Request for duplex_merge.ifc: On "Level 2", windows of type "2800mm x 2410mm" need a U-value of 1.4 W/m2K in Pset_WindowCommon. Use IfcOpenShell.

First a look at what the model holds.

```python
import ifcopenshell
import ifcopenshell.util.element

model = ifcopenshell.open("duplex_merge.ifc")
print(model.schema)
storey = next(s for s in model.by_type("IfcBuildingStorey") if s.Name == "Level 2")
windows = [e for e in ifcopenshell.util.element.get_decomposition(storey) if e.is_a("IfcWindow")]
seen = {}
for e in windows:
    element_type = ifcopenshell.util.element.get_type(e)
    key = (element_type.Name if element_type != e and element_type else None, ifcopenshell.util.element.get_pset(e, "Pset_WindowCommon", "ThermalTransmittance"))
    seen[key] = seen.get(key, 0) + 1
for (name, value), count in sorted(seen.items(), key=str):
    print(count, "x", name, "|", value)
```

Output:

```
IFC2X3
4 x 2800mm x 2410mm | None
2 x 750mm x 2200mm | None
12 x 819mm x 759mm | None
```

```python
import ifcopenshell
import ifcopenshell.api.pset
import ifcopenshell.util.element

model = ifcopenshell.open("duplex_merge.ifc")

storey = next(s for s in model.by_type("IfcBuildingStorey") if s.Name == "Level 2")
windows = [e for e in ifcopenshell.util.element.get_decomposition(storey) if e.is_a("IfcWindow")]

count = 0
for e in windows:
    element_type = ifcopenshell.util.element.get_type(e)
    if element_type in (None, e) or element_type.Name != "2800mm x 2410mm":
        continue
    # add_pset returns the element's existing set when there is one.
    pset = ifcopenshell.api.pset.add_pset(model, product=e, name="Pset_WindowCommon")
    ifcopenshell.api.pset.edit_pset(model, pset=pset, properties={"ThermalTransmittance": 1.4})
    count += 1

print(count, "windows updated")

model.write("duplex_merge_rev.ifc")
```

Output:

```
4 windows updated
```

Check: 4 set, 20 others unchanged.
